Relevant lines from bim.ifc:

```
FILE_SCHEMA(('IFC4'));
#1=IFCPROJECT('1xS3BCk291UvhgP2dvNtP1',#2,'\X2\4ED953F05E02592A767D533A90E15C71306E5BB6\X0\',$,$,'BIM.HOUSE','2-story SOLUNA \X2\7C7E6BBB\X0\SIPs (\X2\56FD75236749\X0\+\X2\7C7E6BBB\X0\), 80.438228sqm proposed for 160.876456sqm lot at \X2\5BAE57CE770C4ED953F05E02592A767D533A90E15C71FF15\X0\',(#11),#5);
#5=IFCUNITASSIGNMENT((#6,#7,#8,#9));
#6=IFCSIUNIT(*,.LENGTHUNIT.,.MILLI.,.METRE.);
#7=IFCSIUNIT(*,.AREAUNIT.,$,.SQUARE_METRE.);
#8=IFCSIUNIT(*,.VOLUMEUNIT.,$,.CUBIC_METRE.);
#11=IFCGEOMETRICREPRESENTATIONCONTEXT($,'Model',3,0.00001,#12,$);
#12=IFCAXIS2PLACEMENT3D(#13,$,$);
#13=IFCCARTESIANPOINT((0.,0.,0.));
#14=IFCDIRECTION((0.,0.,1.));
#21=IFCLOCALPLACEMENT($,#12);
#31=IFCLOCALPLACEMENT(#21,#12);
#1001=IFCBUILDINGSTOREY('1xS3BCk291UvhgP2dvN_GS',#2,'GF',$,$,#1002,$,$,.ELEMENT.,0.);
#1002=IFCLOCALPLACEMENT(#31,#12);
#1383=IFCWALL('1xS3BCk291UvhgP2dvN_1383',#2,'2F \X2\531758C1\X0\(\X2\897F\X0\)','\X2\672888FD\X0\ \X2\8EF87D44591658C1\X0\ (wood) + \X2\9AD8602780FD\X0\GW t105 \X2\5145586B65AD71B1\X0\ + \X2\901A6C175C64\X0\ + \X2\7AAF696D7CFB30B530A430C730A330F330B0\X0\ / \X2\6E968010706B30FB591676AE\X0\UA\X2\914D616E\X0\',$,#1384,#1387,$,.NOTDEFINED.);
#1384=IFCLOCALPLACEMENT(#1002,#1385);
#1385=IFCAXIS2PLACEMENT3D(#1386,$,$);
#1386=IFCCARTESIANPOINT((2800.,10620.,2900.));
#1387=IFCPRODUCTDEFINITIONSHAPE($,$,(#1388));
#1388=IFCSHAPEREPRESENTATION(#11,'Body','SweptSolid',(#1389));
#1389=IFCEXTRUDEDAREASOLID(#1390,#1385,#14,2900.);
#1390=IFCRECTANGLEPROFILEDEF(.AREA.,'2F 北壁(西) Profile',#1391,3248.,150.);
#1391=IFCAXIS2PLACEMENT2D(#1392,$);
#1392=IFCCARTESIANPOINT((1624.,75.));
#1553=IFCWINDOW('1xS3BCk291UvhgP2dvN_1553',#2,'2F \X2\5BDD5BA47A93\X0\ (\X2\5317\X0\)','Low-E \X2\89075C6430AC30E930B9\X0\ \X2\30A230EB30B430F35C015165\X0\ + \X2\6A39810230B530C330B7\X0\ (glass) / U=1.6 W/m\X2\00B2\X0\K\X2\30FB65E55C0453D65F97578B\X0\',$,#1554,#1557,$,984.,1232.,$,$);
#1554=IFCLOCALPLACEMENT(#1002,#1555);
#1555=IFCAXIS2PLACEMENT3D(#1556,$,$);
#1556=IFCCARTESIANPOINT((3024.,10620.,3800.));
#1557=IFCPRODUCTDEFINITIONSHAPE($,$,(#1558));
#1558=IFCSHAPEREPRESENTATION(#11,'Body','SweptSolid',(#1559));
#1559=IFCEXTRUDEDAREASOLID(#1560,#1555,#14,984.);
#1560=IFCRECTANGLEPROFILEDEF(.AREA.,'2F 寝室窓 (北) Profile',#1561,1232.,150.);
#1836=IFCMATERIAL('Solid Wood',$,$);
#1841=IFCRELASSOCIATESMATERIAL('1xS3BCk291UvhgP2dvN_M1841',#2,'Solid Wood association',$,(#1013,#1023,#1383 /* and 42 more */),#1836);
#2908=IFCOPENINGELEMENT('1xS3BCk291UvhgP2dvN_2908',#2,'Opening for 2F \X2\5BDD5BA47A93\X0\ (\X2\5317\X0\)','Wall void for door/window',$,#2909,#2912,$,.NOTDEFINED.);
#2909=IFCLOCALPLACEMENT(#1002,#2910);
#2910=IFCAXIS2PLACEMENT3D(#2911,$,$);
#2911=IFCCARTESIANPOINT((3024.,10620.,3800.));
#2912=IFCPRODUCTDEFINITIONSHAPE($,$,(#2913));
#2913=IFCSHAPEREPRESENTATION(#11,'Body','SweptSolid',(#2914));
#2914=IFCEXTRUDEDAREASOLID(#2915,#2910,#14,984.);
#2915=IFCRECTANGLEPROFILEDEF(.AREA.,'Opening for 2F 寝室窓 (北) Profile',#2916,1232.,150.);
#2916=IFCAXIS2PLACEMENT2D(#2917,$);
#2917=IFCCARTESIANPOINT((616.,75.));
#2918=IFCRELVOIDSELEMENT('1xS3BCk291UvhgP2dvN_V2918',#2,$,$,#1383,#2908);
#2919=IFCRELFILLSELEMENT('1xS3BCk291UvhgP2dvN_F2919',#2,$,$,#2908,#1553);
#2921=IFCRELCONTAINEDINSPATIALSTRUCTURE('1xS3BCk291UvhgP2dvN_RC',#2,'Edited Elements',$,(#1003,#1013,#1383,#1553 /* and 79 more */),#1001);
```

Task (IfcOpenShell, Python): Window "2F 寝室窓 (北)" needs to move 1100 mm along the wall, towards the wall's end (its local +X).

```python
import ifcopenshell
import ifcopenshell.api.geometry
import ifcopenshell.util.placement
import ifcopenshell.util.unit

model = ifcopenshell.open("bim.ifc")
unit_scale = ifcopenshell.util.unit.calculate_unit_scale(model)

window = model.by_guid("1xS3BCk291UvhgP2dvN_1553")
opening = window.FillsVoids[0].RelatingOpeningElement
wall = opening.VoidsElements[0].RelatingBuildingElement

wall_matrix = ifcopenshell.util.placement.get_local_placement(wall.ObjectPlacement)
shift = wall_matrix[:3, 0] * 1.1 / unit_scale
before = ifcopenshell.util.placement.get_local_placement(window.ObjectPlacement)[:3, 3].copy()

# The window is not placed relative to its opening, so move both.
for product in (opening, window):
    matrix = ifcopenshell.util.placement.get_local_placement(product.ObjectPlacement)
    matrix[:3, 3] += shift
    ifcopenshell.api.geometry.edit_object_placement(model, product=product, matrix=matrix, is_si=False)

after = ifcopenshell.util.placement.get_local_placement(window.ObjectPlacement)[:3, 3]
print("window moved by", (after - before).round(3) + 0.0)

model.write("bim_rev.ifc")
```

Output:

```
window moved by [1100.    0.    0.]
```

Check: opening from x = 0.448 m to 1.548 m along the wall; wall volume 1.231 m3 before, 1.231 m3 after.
